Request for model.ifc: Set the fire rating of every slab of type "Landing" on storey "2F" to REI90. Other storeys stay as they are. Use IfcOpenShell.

First a look at what the model holds.

```python
import ifcopenshell
import ifcopenshell.util.element

model = ifcopenshell.open("model.ifc")
print(model.schema)
storey = next(s for s in model.by_type("IfcBuildingStorey") if s.Name == "2F")
slabs = [e for e in ifcopenshell.util.element.get_decomposition(storey) if e.is_a("IfcSlab")]
seen = {}
for e in slabs:
    element_type = ifcopenshell.util.element.get_type(e)
    key = (element_type.Name if element_type != e and element_type else None, ifcopenshell.util.element.get_pset(e, "Pset_SlabCommon", "FireRating"))
    seen[key] = seen.get(key, 0) + 1
for (name, value), count in sorted(seen.items(), key=str):
    print(count, "x", name, "|", value)
```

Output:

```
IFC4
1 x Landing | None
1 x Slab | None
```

```python
import ifcopenshell
import ifcopenshell.api.pset
import ifcopenshell.util.element

model = ifcopenshell.open("model.ifc")

storey = next(s for s in model.by_type("IfcBuildingStorey") if s.Name == "2F")
slabs = [e for e in ifcopenshell.util.element.get_decomposition(storey) if e.is_a("IfcSlab")]

count = 0
for e in slabs:
    element_type = ifcopenshell.util.element.get_type(e)
    if element_type in (None, e) or element_type.Name != "Landing":
        continue
    # add_pset returns the element's existing set when there is one.
    pset = ifcopenshell.api.pset.add_pset(model, product=e, name="Pset_SlabCommon")
    ifcopenshell.api.pset.edit_pset(model, pset=pset, properties={"FireRating": "REI90"})
    count += 1

print(count, "slabs updated")

model.write("model_rev.ifc")
```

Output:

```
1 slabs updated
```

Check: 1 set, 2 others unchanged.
